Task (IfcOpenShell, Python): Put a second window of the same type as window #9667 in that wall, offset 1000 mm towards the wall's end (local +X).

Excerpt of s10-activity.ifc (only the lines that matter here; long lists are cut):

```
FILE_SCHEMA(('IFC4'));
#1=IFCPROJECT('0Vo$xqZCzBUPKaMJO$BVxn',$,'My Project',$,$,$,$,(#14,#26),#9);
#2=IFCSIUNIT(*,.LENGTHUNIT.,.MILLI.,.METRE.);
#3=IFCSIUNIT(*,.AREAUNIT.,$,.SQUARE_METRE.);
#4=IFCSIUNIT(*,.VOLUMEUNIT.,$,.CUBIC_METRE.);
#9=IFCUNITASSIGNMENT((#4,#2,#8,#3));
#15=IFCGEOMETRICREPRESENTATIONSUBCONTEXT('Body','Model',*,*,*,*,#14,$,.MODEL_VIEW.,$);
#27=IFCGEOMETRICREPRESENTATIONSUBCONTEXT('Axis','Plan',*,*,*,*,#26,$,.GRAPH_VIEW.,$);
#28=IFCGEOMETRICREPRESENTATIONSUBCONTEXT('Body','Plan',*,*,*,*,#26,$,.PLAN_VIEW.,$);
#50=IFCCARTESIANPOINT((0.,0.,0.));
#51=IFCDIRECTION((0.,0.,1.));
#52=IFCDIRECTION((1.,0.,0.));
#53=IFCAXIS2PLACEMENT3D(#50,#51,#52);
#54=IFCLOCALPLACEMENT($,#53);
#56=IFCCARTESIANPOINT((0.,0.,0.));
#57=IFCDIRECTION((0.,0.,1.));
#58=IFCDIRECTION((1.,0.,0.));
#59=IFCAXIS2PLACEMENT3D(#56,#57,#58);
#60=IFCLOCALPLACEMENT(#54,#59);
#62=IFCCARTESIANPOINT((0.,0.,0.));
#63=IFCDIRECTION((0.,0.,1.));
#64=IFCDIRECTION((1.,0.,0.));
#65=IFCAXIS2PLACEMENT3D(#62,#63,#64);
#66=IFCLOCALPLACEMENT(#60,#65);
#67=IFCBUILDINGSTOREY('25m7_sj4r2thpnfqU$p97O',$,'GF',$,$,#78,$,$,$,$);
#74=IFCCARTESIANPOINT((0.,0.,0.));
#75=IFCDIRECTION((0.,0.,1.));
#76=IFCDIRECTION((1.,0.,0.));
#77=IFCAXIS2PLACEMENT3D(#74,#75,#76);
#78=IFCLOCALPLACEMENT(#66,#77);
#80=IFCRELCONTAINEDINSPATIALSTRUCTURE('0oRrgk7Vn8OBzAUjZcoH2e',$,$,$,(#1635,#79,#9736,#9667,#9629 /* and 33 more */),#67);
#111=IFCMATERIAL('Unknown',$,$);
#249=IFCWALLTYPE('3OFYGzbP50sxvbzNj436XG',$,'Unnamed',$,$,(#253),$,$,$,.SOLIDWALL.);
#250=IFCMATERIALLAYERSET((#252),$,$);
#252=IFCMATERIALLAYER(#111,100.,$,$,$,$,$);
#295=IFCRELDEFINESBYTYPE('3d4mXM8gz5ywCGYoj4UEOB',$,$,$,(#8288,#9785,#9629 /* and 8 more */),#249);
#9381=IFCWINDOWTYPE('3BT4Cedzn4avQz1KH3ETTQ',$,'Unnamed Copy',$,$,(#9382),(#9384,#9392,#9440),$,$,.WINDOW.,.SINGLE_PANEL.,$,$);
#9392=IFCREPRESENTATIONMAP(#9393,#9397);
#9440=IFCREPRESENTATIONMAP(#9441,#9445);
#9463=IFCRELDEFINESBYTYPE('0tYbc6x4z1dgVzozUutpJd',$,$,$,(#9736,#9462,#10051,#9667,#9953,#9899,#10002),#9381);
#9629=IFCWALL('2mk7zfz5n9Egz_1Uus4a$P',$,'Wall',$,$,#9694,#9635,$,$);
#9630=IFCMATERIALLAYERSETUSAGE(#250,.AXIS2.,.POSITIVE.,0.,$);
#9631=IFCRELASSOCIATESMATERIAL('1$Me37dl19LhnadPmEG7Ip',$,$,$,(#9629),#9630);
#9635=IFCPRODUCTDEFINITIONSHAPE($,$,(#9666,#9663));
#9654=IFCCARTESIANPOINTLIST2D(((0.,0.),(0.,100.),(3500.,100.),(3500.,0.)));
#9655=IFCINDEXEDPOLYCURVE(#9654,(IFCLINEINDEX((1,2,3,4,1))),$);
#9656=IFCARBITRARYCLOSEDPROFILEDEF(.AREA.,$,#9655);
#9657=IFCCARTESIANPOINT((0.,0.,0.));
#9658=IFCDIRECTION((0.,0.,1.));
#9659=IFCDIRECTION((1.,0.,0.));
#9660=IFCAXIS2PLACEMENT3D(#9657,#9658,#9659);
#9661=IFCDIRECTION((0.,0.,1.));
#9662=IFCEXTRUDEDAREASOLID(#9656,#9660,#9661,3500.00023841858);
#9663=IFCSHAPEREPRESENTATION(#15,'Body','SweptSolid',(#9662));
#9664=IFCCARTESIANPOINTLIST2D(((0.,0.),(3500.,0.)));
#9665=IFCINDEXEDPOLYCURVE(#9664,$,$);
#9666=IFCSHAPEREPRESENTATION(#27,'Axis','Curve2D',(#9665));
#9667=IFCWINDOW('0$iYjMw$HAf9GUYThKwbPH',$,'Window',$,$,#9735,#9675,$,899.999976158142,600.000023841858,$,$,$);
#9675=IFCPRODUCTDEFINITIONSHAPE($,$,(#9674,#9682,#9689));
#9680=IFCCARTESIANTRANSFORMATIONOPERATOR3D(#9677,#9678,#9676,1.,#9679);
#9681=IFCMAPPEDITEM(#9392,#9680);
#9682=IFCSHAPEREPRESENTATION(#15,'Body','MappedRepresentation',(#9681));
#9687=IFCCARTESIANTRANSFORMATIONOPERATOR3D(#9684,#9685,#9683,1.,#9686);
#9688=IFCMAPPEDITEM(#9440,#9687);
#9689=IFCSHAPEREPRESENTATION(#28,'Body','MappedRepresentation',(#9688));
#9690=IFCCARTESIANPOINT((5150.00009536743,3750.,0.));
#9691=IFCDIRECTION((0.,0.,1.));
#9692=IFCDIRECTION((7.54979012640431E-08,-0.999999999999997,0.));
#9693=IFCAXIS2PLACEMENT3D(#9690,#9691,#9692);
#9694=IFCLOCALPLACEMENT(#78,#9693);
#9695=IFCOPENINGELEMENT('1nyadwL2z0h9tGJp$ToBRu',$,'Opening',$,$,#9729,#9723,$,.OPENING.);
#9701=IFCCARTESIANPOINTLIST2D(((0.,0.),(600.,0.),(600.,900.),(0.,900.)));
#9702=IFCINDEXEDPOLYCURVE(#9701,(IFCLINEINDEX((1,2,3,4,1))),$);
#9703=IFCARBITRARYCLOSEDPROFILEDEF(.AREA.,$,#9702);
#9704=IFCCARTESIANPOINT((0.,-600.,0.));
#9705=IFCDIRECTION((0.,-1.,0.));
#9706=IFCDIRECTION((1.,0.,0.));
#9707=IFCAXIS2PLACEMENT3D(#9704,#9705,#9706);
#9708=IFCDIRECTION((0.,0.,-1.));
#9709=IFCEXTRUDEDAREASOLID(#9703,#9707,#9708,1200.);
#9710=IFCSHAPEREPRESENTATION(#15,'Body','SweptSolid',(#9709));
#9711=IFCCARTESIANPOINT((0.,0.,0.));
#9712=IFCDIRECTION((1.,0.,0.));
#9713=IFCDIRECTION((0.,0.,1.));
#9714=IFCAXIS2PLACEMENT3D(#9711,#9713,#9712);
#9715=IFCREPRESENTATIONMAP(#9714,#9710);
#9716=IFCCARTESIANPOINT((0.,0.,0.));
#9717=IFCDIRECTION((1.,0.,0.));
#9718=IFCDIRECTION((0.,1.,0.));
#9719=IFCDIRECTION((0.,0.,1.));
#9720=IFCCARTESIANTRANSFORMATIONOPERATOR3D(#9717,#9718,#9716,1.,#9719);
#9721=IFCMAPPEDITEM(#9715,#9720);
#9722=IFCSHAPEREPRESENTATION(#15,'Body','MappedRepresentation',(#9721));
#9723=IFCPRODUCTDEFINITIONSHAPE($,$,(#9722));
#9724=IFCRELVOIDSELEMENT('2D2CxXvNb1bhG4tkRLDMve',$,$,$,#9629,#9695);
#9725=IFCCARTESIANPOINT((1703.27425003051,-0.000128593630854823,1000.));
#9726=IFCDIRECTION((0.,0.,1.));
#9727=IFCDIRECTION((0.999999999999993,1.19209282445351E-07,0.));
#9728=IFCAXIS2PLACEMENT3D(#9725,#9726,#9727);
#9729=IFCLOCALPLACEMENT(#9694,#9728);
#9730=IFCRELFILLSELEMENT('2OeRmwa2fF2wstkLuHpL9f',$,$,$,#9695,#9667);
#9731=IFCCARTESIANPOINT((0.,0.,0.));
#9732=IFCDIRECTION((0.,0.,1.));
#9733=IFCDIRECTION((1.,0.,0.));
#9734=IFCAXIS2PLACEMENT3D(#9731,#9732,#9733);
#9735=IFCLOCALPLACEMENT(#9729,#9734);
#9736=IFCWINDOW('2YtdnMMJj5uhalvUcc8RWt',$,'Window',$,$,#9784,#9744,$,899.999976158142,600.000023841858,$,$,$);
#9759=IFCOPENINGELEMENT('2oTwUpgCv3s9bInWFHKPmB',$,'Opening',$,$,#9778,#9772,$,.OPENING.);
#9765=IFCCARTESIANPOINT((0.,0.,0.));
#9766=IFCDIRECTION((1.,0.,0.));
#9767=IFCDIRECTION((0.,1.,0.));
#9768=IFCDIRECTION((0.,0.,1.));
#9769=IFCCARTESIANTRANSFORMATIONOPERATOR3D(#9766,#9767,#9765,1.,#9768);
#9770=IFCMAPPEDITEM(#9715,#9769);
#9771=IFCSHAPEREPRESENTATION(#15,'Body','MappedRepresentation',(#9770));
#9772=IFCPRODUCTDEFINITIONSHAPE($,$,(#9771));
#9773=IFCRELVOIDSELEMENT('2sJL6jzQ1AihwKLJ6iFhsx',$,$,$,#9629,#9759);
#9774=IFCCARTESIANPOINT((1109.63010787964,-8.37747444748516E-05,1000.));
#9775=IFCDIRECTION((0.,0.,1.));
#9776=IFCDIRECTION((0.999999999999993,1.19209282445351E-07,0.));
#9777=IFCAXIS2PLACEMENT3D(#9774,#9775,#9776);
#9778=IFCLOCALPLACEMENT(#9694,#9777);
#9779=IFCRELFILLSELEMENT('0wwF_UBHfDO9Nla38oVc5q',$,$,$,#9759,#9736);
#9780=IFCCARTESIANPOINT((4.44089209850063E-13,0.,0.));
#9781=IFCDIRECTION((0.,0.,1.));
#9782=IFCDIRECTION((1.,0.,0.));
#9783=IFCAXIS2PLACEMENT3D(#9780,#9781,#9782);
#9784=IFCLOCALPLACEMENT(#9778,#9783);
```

```python
import ifcopenshell
import ifcopenshell.api.feature
import ifcopenshell.api.geometry
import ifcopenshell.api.root
import ifcopenshell.geom
import ifcopenshell.util.element
import ifcopenshell.util.placement
import ifcopenshell.util.shape
import ifcopenshell.util.unit

model = ifcopenshell.open("s10-activity.ifc")
unit_scale = ifcopenshell.util.unit.calculate_unit_scale(model)
settings = ifcopenshell.geom.settings()


def volume(element):
    """Net volume in cubic metres, openings subtracted."""
    shape = ifcopenshell.geom.create_shape(settings, element)
    return ifcopenshell.util.shape.get_volume(shape.geometry)


window = model.by_id(9667)
opening = window.FillsVoids[0].RelatingOpeningElement
wall = opening.VoidsElements[0].RelatingBuildingElement
before = volume(wall)
shift = ifcopenshell.util.placement.get_local_placement(wall.ObjectPlacement)[:3, 0] * 1 / unit_scale

# copy_class copies the void relationship, type, container and properties, but no geometry.
new_opening = ifcopenshell.api.root.copy_class(model, product=opening)
new_opening.Representation = ifcopenshell.util.element.copy_deep(
    model, opening.Representation, exclude=["IfcGeometricRepresentationContext", "IfcRepresentationMap"]
)
new_window = ifcopenshell.api.root.copy_class(model, product=window)
new_window.Representation = ifcopenshell.util.element.copy_deep(
    model, window.Representation, exclude=["IfcGeometricRepresentationContext", "IfcRepresentationMap"]
)
ifcopenshell.api.feature.add_filling(model, opening=new_opening, element=new_window)

for old, new in ((opening, new_opening), (window, new_window)):
    matrix = ifcopenshell.util.placement.get_local_placement(old.ObjectPlacement)
    matrix[:3, 3] += shift
    ifcopenshell.api.geometry.edit_object_placement(model, product=new, matrix=matrix, is_si=False)

after = volume(wall)

print(f"wall volume {before:.3f} -> {after:.3f} m3")

model.write("s10-activity_edited.ifc")
```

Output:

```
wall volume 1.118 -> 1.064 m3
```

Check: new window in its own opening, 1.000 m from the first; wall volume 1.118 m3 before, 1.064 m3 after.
